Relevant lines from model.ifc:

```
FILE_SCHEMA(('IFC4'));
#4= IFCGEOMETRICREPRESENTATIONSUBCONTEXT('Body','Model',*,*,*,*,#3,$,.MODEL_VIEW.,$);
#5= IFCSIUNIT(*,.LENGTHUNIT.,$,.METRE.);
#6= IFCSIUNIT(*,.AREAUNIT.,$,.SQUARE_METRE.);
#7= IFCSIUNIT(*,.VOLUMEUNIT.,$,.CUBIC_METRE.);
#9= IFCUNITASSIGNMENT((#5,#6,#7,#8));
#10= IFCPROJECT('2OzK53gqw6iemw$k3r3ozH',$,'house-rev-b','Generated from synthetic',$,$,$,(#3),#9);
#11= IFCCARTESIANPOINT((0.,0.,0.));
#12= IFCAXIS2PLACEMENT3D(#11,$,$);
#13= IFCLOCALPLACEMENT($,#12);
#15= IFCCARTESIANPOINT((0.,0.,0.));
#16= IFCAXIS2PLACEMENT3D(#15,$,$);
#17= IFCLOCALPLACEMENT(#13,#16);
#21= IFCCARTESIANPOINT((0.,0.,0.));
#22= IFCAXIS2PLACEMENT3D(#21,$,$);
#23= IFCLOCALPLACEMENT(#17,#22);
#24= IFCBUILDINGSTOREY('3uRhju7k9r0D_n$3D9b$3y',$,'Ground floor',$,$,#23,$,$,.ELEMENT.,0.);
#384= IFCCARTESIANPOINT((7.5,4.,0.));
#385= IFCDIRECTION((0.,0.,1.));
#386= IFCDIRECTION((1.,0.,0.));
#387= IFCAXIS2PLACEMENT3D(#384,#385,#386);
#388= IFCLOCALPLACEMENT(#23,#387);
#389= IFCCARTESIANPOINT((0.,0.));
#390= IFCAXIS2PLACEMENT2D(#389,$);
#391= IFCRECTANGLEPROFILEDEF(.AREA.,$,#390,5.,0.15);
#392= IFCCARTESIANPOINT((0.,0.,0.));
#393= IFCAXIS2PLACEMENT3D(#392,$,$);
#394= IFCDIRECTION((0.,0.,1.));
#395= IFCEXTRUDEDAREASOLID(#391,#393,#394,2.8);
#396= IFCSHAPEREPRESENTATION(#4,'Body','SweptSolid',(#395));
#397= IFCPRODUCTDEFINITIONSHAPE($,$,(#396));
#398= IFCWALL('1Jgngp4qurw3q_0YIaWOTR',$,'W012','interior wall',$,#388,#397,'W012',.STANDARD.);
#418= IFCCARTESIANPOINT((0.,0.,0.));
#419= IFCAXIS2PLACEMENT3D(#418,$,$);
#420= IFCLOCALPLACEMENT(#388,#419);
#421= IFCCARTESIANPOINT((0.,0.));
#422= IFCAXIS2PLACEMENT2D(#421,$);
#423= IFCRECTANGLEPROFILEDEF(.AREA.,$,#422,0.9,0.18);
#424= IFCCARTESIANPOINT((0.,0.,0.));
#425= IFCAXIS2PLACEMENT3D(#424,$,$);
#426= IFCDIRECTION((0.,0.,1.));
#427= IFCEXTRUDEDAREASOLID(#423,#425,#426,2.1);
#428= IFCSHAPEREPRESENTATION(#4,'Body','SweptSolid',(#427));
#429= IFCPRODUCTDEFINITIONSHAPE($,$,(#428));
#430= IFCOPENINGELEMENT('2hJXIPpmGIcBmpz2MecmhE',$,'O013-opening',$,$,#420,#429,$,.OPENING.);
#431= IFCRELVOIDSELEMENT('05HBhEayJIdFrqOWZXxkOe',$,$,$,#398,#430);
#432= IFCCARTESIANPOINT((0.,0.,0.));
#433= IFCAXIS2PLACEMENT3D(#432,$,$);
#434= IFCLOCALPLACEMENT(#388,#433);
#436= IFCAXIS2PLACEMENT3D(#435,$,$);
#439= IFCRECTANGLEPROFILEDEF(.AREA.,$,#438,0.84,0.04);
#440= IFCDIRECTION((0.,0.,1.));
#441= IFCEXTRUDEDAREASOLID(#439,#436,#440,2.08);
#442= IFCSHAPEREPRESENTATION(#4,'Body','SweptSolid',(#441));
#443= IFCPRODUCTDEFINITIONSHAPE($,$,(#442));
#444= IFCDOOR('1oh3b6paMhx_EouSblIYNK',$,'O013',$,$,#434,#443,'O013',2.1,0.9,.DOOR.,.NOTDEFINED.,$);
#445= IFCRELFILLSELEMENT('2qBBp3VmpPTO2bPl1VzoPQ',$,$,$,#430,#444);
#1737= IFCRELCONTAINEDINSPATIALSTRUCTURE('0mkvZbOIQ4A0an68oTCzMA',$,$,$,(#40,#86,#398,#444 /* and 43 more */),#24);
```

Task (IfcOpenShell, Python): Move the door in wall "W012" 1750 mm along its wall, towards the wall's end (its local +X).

```python
import ifcopenshell
import ifcopenshell.api.geometry
import ifcopenshell.util.placement
import ifcopenshell.util.unit

model = ifcopenshell.open("model.ifc")
unit_scale = ifcopenshell.util.unit.calculate_unit_scale(model)

door = model.by_guid("1oh3b6paMhx_EouSblIYNK")
opening = door.FillsVoids[0].RelatingOpeningElement
wall = opening.VoidsElements[0].RelatingBuildingElement

wall_matrix = ifcopenshell.util.placement.get_local_placement(wall.ObjectPlacement)
shift = wall_matrix[:3, 0] * 1.75 / unit_scale
before = ifcopenshell.util.placement.get_local_placement(door.ObjectPlacement)[:3, 3].copy()

# The door is not placed relative to its opening, so move both.
for product in (opening, door):
    matrix = ifcopenshell.util.placement.get_local_placement(product.ObjectPlacement)
    matrix[:3, 3] += shift
    ifcopenshell.api.geometry.edit_object_placement(model, product=product, matrix=matrix, is_si=False)

after = ifcopenshell.util.placement.get_local_placement(door.ObjectPlacement)[:3, 3]
print("door moved by", (after - before).round(3) + 0.0)

model.write("model_updated.ifc")
```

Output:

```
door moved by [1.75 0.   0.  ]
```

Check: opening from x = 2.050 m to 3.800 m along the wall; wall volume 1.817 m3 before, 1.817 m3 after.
